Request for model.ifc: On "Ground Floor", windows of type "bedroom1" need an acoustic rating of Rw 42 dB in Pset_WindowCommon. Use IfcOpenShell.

First a look at what the model holds.

```python
import ifcopenshell
import ifcopenshell.util.element

model = ifcopenshell.open("model.ifc")
print(model.schema)
storey = next(s for s in model.by_type("IfcBuildingStorey") if s.Name == "Ground Floor")
windows = [e for e in ifcopenshell.util.element.get_decomposition(storey) if e.is_a("IfcWindow")]
seen = {}
for e in windows:
    element_type = ifcopenshell.util.element.get_type(e)
    key = (element_type.Name if element_type != e and element_type else None, ifcopenshell.util.element.get_pset(e, "Pset_WindowCommon", "AcousticRating"))
    seen[key] = seen.get(key, 0) + 1
for (name, value), count in sorted(seen.items(), key=str):
    print(count, "x", name, "|", value)
```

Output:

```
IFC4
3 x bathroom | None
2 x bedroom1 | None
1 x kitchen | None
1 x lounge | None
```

```python
import ifcopenshell
import ifcopenshell.api.pset
import ifcopenshell.util.element

model = ifcopenshell.open("model.ifc")

storey = next(s for s in model.by_type("IfcBuildingStorey") if s.Name == "Ground Floor")
windows = [e for e in ifcopenshell.util.element.get_decomposition(storey) if e.is_a("IfcWindow")]

count = 0
for e in windows:
    element_type = ifcopenshell.util.element.get_type(e)
    if element_type in (None, e) or element_type.Name != "bedroom1":
        continue
    # add_pset returns the element's existing set when there is one.
    pset = ifcopenshell.api.pset.add_pset(model, product=e, name="Pset_WindowCommon")
    ifcopenshell.api.pset.edit_pset(model, pset=pset, properties={"AcousticRating": "Rw 42 dB"})
    count += 1

print(count, "windows updated")

model.write("model_updated.ifc")
```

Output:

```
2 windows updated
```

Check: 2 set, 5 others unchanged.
